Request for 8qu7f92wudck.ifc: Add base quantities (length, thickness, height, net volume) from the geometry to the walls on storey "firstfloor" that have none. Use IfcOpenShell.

First a look at what the model holds.

```python
import ifcopenshell
import ifcopenshell.util.element
import ifcopenshell.util.unit

model = ifcopenshell.open("8qu7f92wudck.ifc")
print(model.schema)
for unit_type in ("LENGTHUNIT", "AREAUNIT", "VOLUMEUNIT"):
    print(unit_type, ifcopenshell.util.unit.calculate_unit_scale(model, unit_type))
storey = next(s for s in model.by_type("IfcBuildingStorey") if s.Name == "firstfloor")
walls = [e for e in ifcopenshell.util.element.get_decomposition(storey) if e.is_a("IfcWall")]
for e in sorted(walls, key=lambda e: e.id()):
    print(e.id(), e.is_a(), e.Name, list(ifcopenshell.util.element.get_psets(e, qtos_only=True)), sep=" | ")
```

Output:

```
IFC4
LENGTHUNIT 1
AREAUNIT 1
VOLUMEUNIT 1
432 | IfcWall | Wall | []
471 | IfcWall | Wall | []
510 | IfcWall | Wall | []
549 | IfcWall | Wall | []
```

```python
import ifcopenshell
import ifcopenshell.api.pset
import ifcopenshell.geom
import ifcopenshell.util.element
import ifcopenshell.util.shape
import ifcopenshell.util.unit

model = ifcopenshell.open("8qu7f92wudck.ifc")
unit_scale = ifcopenshell.util.unit.calculate_unit_scale(model)
volume_scale = ifcopenshell.util.unit.calculate_unit_scale(model, "VOLUMEUNIT")
settings = ifcopenshell.geom.settings()

storey = next(s for s in model.by_type("IfcBuildingStorey") if s.Name == "firstfloor")
walls = [e for e in ifcopenshell.util.element.get_decomposition(storey) if e.is_a("IfcWall")]

for e in sorted(walls, key=lambda e: e.id()):
    if ifcopenshell.util.element.get_psets(e, qtos_only=True, should_inherit=False):
        continue
    # Geometry comes back in metres, in the element's own axes.
    shape = ifcopenshell.geom.create_shape(settings, e)
    values = {
        "Length": ifcopenshell.util.shape.get_x(shape.geometry) / unit_scale,
        "Width": ifcopenshell.util.shape.get_y(shape.geometry) / unit_scale,
        "Height": ifcopenshell.util.shape.get_z(shape.geometry) / unit_scale,
        "NetVolume": ifcopenshell.util.shape.get_volume(shape.geometry) / volume_scale,
    }
    qto = ifcopenshell.api.pset.add_qto(model, product=e, name="Qto_WallBaseQuantities")
    ifcopenshell.api.pset.edit_qto(model, qto=qto, properties=values)
    print(e.id(), {k: round(v, 3) for k, v in values.items()})

model.write("8qu7f92wudck_v2.ifc")
```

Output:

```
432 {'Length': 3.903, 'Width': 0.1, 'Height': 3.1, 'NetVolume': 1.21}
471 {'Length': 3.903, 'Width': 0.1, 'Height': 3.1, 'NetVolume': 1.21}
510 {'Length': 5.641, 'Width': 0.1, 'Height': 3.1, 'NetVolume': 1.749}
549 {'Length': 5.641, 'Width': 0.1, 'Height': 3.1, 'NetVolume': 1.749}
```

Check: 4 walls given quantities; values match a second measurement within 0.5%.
